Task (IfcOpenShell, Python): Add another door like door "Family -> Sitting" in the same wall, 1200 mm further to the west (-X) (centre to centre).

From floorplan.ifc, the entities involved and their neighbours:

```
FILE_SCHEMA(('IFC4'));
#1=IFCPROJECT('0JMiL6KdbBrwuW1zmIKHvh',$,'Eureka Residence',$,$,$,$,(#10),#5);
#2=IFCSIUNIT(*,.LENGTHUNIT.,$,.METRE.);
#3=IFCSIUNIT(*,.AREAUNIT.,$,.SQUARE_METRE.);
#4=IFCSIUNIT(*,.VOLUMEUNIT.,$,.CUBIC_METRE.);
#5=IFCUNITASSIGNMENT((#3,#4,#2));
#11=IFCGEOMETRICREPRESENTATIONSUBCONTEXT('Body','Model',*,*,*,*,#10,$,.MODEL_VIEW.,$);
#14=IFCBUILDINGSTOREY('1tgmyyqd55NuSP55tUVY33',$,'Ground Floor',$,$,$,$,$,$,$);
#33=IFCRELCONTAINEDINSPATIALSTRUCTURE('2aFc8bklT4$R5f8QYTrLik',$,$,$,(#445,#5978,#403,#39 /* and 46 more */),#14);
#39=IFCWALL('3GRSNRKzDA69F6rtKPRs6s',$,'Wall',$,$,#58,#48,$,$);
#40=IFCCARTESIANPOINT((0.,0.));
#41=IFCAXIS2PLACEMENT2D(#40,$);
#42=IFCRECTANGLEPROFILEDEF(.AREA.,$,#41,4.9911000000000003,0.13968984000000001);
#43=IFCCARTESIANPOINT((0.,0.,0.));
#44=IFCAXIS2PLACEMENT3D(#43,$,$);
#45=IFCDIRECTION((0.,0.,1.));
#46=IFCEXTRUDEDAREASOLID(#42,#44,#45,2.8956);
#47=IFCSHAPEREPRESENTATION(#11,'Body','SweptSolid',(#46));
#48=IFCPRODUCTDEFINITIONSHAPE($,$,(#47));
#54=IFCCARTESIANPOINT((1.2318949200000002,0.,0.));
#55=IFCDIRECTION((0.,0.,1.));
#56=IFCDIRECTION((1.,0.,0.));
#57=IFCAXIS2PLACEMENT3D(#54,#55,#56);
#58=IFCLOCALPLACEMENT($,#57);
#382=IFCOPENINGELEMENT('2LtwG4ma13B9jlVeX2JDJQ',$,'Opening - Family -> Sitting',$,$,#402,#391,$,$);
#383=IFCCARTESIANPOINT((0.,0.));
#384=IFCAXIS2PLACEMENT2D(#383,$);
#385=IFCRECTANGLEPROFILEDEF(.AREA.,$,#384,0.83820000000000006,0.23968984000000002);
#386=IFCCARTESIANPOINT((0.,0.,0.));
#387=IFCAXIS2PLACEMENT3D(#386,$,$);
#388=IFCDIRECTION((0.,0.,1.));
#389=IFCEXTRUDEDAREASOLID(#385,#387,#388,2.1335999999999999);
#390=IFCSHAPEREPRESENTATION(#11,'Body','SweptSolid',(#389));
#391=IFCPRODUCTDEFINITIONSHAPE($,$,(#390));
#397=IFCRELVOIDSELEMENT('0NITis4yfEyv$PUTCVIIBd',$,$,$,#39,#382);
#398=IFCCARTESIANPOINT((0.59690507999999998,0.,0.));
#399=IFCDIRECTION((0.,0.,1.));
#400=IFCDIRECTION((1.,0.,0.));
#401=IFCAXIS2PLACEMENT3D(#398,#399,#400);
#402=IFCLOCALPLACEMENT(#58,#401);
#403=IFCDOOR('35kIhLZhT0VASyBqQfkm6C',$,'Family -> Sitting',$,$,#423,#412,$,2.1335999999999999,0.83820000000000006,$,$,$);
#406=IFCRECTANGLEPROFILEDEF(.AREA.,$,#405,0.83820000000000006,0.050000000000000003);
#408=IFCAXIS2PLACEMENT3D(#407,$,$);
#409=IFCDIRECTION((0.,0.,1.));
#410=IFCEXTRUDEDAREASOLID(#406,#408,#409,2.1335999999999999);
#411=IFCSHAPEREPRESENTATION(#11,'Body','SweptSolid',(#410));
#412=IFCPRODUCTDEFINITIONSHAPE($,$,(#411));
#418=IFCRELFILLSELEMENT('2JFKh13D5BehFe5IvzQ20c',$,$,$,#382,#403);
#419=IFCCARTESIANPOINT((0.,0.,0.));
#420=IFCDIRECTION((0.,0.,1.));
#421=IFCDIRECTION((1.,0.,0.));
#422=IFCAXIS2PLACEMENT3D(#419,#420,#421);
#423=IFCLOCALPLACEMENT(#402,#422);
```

```python
import ifcopenshell
import ifcopenshell.api.feature
import ifcopenshell.api.geometry
import ifcopenshell.api.root
import ifcopenshell.geom
import ifcopenshell.util.element
import ifcopenshell.util.placement
import ifcopenshell.util.shape

model = ifcopenshell.open("floorplan.ifc")
settings = ifcopenshell.geom.settings()


def volume(element):
    """Net volume in cubic metres, openings subtracted."""
    shape = ifcopenshell.geom.create_shape(settings, element)
    return ifcopenshell.util.shape.get_volume(shape.geometry)


door = model.by_guid("35kIhLZhT0VASyBqQfkm6C")
opening = door.FillsVoids[0].RelatingOpeningElement
wall = opening.VoidsElements[0].RelatingBuildingElement
before = volume(wall)
shift = ifcopenshell.util.placement.get_local_placement(wall.ObjectPlacement)[:3, 0] * -1.2

# copy_class copies the void relationship, type, container and properties, but no geometry.
new_opening = ifcopenshell.api.root.copy_class(model, product=opening)
new_opening.Representation = ifcopenshell.util.element.copy_deep(
    model, opening.Representation, exclude=["IfcGeometricRepresentationContext", "IfcRepresentationMap"]
)
new_door = ifcopenshell.api.root.copy_class(model, product=door)
new_door.Representation = ifcopenshell.util.element.copy_deep(
    model, door.Representation, exclude=["IfcGeometricRepresentationContext", "IfcRepresentationMap"]
)
ifcopenshell.api.feature.add_filling(model, opening=new_opening, element=new_door)

for old, new in ((opening, new_opening), (door, new_door)):
    matrix = ifcopenshell.util.placement.get_local_placement(old.ObjectPlacement)
    matrix[:3, 3] += shift
    ifcopenshell.api.geometry.edit_object_placement(model, product=new, matrix=matrix, is_si=False)

after = volume(wall)

print(f"wall volume {before:.3f} -> {after:.3f} m3")

model.write("floorplan-out.ifc")
```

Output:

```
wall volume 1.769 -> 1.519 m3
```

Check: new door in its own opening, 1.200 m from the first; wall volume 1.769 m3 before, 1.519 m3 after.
